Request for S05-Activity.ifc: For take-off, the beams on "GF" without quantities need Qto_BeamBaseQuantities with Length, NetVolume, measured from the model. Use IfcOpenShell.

First a look at what the model holds.

```python
import ifcopenshell
import ifcopenshell.util.element
import ifcopenshell.util.unit

model = ifcopenshell.open("S05-Activity.ifc")
print(model.schema)
for unit_type in ("LENGTHUNIT", "AREAUNIT", "VOLUMEUNIT"):
    print(unit_type, ifcopenshell.util.unit.calculate_unit_scale(model, unit_type))
storey = next(s for s in model.by_type("IfcBuildingStorey") if s.Name == "GF")
beams = [e for e in ifcopenshell.util.element.get_decomposition(storey) if e.is_a("IfcBeam")]
for e in sorted(beams, key=lambda e: e.id()):
    print(e.id(), e.is_a(), e.Name, list(ifcopenshell.util.element.get_psets(e, qtos_only=True)), sep=" | ")
```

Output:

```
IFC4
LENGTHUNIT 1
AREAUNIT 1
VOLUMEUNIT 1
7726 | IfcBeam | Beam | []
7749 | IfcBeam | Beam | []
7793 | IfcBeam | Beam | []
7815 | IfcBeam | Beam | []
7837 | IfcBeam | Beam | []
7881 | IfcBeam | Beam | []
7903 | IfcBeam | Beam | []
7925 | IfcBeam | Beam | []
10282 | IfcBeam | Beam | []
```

```python
import ifcopenshell
import ifcopenshell.api.pset
import ifcopenshell.geom
import ifcopenshell.util.element
import ifcopenshell.util.shape
import ifcopenshell.util.unit

model = ifcopenshell.open("S05-Activity.ifc")
unit_scale = ifcopenshell.util.unit.calculate_unit_scale(model)
volume_scale = ifcopenshell.util.unit.calculate_unit_scale(model, "VOLUMEUNIT")
settings = ifcopenshell.geom.settings()

storey = next(s for s in model.by_type("IfcBuildingStorey") if s.Name == "GF")
beams = [e for e in ifcopenshell.util.element.get_decomposition(storey) if e.is_a("IfcBeam")]

for e in sorted(beams, key=lambda e: e.id()):
    if ifcopenshell.util.element.get_psets(e, qtos_only=True, should_inherit=False):
        continue
    # Geometry comes back in metres, in the element's own axes.
    shape = ifcopenshell.geom.create_shape(settings, e)
    values = {
        "Length": ifcopenshell.util.shape.get_max_xyz(shape.geometry) / unit_scale,
        "NetVolume": ifcopenshell.util.shape.get_volume(shape.geometry) / volume_scale,
    }
    qto = ifcopenshell.api.pset.add_qto(model, product=e, name="Qto_BeamBaseQuantities")
    ifcopenshell.api.pset.edit_qto(model, qto=qto, properties=values)
    print(e.id(), {k: round(v, 3) for k, v in values.items()})

model.write("S05-Activity_edited.ifc")
```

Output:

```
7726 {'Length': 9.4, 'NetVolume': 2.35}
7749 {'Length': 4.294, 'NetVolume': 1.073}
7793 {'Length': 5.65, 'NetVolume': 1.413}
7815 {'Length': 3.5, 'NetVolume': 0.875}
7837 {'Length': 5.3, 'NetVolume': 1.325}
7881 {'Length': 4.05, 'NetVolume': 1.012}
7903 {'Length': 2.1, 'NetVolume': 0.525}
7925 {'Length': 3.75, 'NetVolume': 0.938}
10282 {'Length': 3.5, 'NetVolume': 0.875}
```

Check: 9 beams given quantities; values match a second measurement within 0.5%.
